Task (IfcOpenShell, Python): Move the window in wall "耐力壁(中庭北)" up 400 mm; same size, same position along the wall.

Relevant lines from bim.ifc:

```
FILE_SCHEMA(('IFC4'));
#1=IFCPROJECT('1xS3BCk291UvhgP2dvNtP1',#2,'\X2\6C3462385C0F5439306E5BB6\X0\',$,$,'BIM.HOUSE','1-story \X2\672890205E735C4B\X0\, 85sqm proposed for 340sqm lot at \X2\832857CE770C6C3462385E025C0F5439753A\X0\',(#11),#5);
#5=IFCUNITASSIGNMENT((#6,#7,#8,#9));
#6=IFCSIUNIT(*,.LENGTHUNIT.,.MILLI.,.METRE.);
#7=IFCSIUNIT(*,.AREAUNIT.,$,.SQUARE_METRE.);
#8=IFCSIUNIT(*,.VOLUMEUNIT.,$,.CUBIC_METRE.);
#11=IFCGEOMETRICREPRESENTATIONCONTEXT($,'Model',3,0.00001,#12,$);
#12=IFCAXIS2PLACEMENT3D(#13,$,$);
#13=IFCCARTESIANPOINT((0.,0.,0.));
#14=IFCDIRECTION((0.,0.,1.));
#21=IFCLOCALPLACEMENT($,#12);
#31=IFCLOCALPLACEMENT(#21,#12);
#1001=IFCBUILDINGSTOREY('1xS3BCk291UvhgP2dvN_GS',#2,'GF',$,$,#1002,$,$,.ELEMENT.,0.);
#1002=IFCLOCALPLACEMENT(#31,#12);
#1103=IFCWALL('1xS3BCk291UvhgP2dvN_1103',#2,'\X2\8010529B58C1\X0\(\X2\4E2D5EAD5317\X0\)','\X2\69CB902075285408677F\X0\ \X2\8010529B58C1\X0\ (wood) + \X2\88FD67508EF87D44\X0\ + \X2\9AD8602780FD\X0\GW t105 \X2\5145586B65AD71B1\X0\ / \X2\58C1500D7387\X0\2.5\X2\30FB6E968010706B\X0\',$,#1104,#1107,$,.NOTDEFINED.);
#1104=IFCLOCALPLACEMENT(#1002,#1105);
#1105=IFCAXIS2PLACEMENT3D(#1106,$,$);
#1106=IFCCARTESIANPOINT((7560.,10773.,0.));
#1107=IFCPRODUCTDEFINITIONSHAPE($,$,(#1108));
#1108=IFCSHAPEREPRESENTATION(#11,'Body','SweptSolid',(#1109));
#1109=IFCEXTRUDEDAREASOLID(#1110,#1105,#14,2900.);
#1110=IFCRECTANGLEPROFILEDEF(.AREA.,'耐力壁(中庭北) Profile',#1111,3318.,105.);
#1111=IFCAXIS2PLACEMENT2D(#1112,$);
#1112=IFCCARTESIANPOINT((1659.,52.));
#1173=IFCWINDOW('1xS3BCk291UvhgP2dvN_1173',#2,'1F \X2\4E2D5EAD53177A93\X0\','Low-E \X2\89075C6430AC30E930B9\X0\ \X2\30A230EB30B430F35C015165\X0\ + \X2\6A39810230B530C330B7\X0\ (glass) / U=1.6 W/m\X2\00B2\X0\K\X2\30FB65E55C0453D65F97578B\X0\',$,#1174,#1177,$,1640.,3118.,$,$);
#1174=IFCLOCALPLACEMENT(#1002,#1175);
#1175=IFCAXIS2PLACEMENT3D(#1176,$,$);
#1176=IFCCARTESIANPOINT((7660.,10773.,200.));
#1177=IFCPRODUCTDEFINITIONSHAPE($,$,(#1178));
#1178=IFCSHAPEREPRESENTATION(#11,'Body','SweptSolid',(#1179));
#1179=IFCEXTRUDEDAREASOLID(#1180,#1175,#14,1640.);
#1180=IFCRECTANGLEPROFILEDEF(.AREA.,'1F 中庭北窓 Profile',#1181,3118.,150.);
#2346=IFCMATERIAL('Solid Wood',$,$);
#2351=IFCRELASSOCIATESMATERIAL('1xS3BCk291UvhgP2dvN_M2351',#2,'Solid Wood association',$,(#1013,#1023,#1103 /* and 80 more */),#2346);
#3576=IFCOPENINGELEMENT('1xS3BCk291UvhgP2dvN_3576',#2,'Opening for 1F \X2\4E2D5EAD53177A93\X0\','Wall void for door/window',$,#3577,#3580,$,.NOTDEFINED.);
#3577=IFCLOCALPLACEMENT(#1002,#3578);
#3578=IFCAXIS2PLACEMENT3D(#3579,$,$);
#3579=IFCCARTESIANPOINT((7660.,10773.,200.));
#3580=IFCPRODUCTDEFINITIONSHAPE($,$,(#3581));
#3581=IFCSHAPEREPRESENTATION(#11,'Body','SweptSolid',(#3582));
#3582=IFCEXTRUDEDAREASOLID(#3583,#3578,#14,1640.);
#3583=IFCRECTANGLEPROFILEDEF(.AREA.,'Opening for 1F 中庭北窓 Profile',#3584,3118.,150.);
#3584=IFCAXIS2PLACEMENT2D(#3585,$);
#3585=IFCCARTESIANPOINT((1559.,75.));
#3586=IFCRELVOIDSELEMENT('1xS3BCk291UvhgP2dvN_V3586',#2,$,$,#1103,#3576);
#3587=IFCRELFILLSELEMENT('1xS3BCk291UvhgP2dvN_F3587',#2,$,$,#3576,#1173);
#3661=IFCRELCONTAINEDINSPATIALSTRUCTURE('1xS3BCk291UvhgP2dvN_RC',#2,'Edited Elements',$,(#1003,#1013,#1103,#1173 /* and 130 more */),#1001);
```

```python
import numpy as np
import ifcopenshell
import ifcopenshell.api.geometry
import ifcopenshell.util.placement
import ifcopenshell.util.unit

model = ifcopenshell.open("bim.ifc")
unit_scale = ifcopenshell.util.unit.calculate_unit_scale(model)

window = model.by_guid("1xS3BCk291UvhgP2dvN_1173")
opening = window.FillsVoids[0].RelatingOpeningElement
dz = 0.4 / unit_scale

shift = np.array([0.0, 0.0, dz])
# The window is not placed relative to its opening, so move both.
for product in (opening, window):
    matrix = ifcopenshell.util.placement.get_local_placement(product.ObjectPlacement)
    matrix[:3, 3] += shift
    ifcopenshell.api.geometry.edit_object_placement(model, product=product, matrix=matrix, is_si=False)

print(f"moved by {dz * unit_scale:+.3f} m")

model.write("bim-out.ifc")
```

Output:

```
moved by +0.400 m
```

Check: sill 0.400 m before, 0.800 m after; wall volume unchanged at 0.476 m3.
